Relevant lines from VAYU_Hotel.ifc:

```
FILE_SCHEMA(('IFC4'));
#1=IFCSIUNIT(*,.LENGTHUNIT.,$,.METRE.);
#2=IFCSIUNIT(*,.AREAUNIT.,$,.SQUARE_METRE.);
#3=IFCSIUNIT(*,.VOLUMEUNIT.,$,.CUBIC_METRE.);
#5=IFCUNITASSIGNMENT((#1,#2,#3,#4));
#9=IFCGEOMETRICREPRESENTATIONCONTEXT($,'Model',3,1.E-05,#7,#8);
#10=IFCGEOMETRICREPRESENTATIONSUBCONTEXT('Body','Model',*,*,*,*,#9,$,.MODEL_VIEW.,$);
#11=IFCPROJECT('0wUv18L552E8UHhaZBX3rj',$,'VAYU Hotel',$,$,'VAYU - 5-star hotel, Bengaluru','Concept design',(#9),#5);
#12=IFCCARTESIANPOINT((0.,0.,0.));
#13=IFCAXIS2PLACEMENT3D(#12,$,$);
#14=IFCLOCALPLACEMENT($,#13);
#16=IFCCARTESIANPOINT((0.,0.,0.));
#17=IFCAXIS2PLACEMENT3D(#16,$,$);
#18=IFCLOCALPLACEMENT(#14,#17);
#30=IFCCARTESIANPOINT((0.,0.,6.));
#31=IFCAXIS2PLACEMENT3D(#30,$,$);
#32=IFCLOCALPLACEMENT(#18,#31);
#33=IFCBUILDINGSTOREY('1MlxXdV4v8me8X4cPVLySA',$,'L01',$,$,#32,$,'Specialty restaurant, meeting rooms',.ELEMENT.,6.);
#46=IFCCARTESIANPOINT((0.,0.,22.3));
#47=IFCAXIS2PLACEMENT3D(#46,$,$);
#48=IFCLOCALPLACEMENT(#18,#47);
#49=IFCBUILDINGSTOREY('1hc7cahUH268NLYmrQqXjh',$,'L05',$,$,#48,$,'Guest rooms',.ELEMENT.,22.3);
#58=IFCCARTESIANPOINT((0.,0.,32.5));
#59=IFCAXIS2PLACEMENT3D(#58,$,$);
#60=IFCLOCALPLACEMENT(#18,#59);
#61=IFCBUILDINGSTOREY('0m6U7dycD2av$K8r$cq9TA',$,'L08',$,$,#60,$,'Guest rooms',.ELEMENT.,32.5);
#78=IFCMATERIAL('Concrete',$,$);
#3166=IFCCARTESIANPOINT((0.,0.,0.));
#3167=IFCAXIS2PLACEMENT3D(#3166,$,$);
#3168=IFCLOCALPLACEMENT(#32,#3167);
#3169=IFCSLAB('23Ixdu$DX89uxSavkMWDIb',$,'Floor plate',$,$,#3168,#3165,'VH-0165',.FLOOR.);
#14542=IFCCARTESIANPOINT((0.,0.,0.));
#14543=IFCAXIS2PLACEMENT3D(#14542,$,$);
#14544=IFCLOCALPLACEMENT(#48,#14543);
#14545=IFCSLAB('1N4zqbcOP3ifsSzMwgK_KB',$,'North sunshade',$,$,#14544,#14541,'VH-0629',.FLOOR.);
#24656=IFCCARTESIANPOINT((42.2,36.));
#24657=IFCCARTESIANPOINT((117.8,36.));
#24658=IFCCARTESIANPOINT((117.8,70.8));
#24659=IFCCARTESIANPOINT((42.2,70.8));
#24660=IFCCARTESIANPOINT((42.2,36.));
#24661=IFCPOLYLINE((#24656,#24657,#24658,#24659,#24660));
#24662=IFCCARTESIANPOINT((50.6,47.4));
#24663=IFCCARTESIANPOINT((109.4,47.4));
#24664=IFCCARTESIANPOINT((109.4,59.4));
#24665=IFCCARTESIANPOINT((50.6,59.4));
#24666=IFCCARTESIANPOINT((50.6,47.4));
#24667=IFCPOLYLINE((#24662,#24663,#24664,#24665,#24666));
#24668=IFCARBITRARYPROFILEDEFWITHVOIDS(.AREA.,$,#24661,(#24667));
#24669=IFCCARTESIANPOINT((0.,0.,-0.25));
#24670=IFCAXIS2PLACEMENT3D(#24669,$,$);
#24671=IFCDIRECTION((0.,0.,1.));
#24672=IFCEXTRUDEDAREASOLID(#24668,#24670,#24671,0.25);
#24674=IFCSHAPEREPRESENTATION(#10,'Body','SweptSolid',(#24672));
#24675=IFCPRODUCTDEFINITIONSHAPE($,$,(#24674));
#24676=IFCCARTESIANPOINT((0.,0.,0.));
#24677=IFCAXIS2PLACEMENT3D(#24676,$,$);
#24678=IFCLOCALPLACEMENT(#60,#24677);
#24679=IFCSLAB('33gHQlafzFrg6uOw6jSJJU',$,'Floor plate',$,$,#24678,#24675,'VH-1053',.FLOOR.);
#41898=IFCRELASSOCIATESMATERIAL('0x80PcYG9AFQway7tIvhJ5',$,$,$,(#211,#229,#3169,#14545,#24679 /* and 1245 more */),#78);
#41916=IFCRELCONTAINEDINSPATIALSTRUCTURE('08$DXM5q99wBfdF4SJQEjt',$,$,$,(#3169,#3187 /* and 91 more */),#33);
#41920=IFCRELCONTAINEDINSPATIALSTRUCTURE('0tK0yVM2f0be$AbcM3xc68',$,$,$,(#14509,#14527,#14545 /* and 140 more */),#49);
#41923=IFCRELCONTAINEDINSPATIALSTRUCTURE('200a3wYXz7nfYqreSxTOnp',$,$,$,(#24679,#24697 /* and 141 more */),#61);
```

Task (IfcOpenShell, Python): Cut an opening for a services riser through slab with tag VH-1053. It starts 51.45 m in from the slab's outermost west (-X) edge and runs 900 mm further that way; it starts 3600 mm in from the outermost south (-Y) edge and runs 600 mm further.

```python
import numpy as np
import ifcopenshell
import ifcopenshell.api.feature
import ifcopenshell.api.geometry
import ifcopenshell.api.root
import ifcopenshell.geom
import ifcopenshell.util.placement
import ifcopenshell.util.representation
import ifcopenshell.util.shape
import ifcopenshell.util.unit

model = ifcopenshell.open("VAYU_Hotel.ifc")
unit_scale = ifcopenshell.util.unit.calculate_unit_scale(model)
settings = ifcopenshell.geom.settings()


def volume(element):
    """Net volume in cubic metres, openings subtracted."""
    shape = ifcopenshell.geom.create_shape(settings, element)
    return ifcopenshell.util.shape.get_volume(shape.geometry)


slab = model.by_guid("33gHQlafzFrg6uOw6jSJJU")
before = volume(slab)

# Extent in the slab's own axes, in metres. The edges named are its -X and -Y sides.
slab_shape = ifcopenshell.geom.create_shape(settings, slab)
vertices = ifcopenshell.util.shape.get_vertices(slab_shape.geometry)
x_min, y_min, bottom = vertices.min(axis=0)
top = vertices[:, 2].max()

opening = ifcopenshell.api.root.create_entity(model, ifc_class="IfcOpeningElement", name="Services riser opening", predefined_type="OPENING")
context = ifcopenshell.util.representation.get_context(model, "Model", "Body", "MODEL_VIEW")
width, depth = 0.9, 0.6
outline = [(0.0, 0.0), (width, 0.0), (width, depth), (0.0, depth), (0.0, 0.0)]
# Overshoot both faces by 50 mm so the cut is clean.
shape = ifcopenshell.api.geometry.add_slab_representation(
    model, context=context, depth=top - bottom + 0.1, polyline=outline
)
ifcopenshell.api.geometry.assign_representation(model, product=opening, representation=shape)

matrix = ifcopenshell.util.placement.get_local_placement(slab.ObjectPlacement)
matrix[:, 3] = matrix @ np.append(np.array([x_min + 51.45, y_min + 3.6, bottom - 0.05]) / unit_scale, 1.0)
ifcopenshell.api.geometry.edit_object_placement(model, product=opening, matrix=matrix, is_si=False)
ifcopenshell.api.feature.add_feature(model, feature=opening, element=slab)

after = volume(slab)

print(f"slab volume {before:.3f} -> {after:.3f} m3")

model.write("VAYU_Hotel_edited.ifc")
```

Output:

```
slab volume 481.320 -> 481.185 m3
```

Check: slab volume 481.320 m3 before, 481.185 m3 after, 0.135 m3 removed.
